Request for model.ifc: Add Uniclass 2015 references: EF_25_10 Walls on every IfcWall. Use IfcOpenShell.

First a look at what the model holds.

```python
import ifcopenshell

model = ifcopenshell.open("model.ifc")
print(model.schema)
print("classifications:", [c.Name for c in model.by_type("IfcClassification")])
for ifc_class in ("IfcDoor", "IfcRoof", "IfcStair", "IfcWall", "IfcWindow"):
    print(ifc_class, len(model.by_type(ifc_class)))
```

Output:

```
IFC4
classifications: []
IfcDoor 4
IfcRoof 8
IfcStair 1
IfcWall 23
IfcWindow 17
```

```python
import ifcopenshell
import ifcopenshell.api.classification

model = ifcopenshell.open("model.ifc")

system = ifcopenshell.api.classification.add_classification(model, classification="Uniclass 2015")

codes = {
    "IfcWall": ("EF_25_10", "Walls"),
}
for ifc_class, (code, name) in codes.items():
    products = model.by_type(ifc_class)
    ifcopenshell.api.classification.add_reference(
        model, products=products, classification=system, identification=code, name=name
    )
    print(code, len(products))

model.write("model-out.ifc")
```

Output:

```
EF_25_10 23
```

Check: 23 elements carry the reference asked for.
